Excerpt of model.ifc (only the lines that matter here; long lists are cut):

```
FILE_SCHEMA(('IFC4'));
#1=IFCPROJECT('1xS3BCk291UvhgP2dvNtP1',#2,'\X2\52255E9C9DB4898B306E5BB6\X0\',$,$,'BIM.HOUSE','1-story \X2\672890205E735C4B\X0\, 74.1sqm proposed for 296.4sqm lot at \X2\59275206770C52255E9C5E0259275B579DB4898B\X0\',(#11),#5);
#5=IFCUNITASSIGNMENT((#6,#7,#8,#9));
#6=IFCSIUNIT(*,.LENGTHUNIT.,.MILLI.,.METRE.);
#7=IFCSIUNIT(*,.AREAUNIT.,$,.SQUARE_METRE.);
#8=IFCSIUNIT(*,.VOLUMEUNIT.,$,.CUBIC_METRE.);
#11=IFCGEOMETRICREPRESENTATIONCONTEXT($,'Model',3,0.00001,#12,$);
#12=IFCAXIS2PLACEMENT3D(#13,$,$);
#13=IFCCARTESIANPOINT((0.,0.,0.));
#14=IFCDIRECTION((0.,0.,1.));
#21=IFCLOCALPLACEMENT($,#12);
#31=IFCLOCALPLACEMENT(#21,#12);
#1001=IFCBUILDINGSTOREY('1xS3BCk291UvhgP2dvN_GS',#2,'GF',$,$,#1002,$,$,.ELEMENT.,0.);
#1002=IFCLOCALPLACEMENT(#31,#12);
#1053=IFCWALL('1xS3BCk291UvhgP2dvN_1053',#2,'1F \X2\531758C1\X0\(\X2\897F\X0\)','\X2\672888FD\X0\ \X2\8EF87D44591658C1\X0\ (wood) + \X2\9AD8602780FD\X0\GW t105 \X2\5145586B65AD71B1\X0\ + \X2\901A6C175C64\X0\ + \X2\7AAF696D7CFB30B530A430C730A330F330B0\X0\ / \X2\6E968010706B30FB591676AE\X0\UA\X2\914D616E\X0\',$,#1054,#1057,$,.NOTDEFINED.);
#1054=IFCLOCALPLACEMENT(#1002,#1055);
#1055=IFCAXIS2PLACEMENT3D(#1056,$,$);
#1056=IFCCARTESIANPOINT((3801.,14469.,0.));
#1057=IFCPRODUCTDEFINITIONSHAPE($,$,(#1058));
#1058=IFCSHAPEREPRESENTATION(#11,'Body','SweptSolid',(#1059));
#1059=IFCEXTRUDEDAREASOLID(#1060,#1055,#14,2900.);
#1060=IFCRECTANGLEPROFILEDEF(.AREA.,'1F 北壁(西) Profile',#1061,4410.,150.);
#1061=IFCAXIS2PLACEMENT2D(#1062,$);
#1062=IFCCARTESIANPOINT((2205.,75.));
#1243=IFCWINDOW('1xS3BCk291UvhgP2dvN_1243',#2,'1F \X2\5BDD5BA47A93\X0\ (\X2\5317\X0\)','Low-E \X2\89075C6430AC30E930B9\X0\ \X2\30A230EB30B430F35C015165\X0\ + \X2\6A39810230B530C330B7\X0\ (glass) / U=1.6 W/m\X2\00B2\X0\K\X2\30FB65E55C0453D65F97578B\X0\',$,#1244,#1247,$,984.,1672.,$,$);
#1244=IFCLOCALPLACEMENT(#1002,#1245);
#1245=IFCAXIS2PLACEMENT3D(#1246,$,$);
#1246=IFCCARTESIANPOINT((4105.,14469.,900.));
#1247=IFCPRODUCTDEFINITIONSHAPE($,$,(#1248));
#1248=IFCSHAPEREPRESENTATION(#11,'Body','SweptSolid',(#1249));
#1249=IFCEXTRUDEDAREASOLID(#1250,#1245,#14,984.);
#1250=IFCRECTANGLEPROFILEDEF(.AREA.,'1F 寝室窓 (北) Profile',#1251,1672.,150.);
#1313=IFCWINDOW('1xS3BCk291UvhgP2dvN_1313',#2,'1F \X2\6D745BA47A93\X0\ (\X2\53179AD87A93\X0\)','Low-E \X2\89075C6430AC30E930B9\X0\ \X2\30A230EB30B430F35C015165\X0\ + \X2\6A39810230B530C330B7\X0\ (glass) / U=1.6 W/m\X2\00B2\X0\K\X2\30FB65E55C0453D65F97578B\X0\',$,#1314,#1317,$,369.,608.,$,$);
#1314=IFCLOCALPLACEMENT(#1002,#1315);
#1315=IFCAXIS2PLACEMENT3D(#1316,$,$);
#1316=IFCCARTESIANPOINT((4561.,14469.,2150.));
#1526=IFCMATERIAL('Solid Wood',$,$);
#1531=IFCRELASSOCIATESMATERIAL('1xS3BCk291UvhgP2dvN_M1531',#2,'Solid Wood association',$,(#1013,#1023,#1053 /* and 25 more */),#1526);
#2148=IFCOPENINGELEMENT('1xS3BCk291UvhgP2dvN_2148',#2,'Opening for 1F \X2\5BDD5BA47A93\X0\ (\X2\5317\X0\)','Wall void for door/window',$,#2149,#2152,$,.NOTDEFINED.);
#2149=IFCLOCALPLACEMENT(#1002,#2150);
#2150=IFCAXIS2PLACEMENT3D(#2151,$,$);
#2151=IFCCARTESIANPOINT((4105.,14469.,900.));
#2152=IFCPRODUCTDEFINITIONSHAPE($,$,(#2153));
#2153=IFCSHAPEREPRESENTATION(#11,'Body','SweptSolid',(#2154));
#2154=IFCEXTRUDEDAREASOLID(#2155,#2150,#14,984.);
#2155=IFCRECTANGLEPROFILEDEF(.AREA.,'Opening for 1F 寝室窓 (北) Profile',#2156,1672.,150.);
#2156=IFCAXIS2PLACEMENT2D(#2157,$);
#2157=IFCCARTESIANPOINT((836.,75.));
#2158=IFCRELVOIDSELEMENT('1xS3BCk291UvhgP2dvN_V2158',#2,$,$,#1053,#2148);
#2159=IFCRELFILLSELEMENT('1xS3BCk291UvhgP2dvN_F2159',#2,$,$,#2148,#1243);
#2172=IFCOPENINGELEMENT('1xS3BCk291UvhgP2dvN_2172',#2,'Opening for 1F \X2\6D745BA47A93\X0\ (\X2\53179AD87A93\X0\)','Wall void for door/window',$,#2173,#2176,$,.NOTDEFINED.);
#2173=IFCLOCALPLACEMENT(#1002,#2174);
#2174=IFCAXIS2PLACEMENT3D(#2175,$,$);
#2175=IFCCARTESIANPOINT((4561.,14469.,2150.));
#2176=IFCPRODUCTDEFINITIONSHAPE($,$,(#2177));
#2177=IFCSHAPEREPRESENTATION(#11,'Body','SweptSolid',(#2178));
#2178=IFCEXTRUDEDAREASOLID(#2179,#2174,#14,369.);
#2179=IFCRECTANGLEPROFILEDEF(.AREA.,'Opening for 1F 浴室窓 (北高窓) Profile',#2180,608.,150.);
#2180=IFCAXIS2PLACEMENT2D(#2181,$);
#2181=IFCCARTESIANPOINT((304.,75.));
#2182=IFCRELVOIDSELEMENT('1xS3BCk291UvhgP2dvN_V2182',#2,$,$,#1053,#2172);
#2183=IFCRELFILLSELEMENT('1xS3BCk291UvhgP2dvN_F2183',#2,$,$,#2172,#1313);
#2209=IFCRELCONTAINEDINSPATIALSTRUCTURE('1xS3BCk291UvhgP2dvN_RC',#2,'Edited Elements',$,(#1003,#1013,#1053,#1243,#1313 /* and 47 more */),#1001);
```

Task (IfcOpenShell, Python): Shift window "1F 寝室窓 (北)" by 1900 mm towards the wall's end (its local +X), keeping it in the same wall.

```python
import ifcopenshell
import ifcopenshell.api.geometry
import ifcopenshell.util.placement
import ifcopenshell.util.unit

model = ifcopenshell.open("model.ifc")
unit_scale = ifcopenshell.util.unit.calculate_unit_scale(model)

window = model.by_guid("1xS3BCk291UvhgP2dvN_1243")
opening = window.FillsVoids[0].RelatingOpeningElement
wall = opening.VoidsElements[0].RelatingBuildingElement

wall_matrix = ifcopenshell.util.placement.get_local_placement(wall.ObjectPlacement)
shift = wall_matrix[:3, 0] * 1.9 / unit_scale
before = ifcopenshell.util.placement.get_local_placement(window.ObjectPlacement)[:3, 3].copy()

# The window is not placed relative to its opening, so move both.
for product in (opening, window):
    matrix = ifcopenshell.util.placement.get_local_placement(product.ObjectPlacement)
    matrix[:3, 3] += shift
    ifcopenshell.api.geometry.edit_object_placement(model, product=product, matrix=matrix, is_si=False)

after = ifcopenshell.util.placement.get_local_placement(window.ObjectPlacement)[:3, 3]
print("window moved by", (after - before).round(3) + 0.0)

model.write("model-out.ifc")
```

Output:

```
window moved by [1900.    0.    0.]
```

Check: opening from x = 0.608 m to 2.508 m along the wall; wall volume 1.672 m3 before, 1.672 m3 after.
